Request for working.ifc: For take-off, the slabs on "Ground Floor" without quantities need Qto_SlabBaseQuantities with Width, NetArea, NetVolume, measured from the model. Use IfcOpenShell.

First a look at what the model holds.

```python
import ifcopenshell
import ifcopenshell.util.element
import ifcopenshell.util.unit

model = ifcopenshell.open("working.ifc")
print(model.schema)
for unit_type in ("LENGTHUNIT", "AREAUNIT", "VOLUMEUNIT"):
    print(unit_type, ifcopenshell.util.unit.calculate_unit_scale(model, unit_type))
storey = next(s for s in model.by_type("IfcBuildingStorey") if s.Name == "Ground Floor")
slabs = [e for e in ifcopenshell.util.element.get_decomposition(storey) if e.is_a("IfcSlab")]
for e in sorted(slabs, key=lambda e: e.id()):
    print(e.id(), e.is_a(), e.Name, list(ifcopenshell.util.element.get_psets(e, qtos_only=True)), sep=" | ")
```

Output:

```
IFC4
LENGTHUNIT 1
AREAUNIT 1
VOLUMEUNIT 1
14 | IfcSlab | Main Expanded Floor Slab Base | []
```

```python
import ifcopenshell
import ifcopenshell.api.pset
import ifcopenshell.geom
import ifcopenshell.util.element
import ifcopenshell.util.shape
import ifcopenshell.util.unit

model = ifcopenshell.open("working.ifc")
unit_scale = ifcopenshell.util.unit.calculate_unit_scale(model)
area_scale = ifcopenshell.util.unit.calculate_unit_scale(model, "AREAUNIT")
volume_scale = ifcopenshell.util.unit.calculate_unit_scale(model, "VOLUMEUNIT")
settings = ifcopenshell.geom.settings()

storey = next(s for s in model.by_type("IfcBuildingStorey") if s.Name == "Ground Floor")
slabs = [e for e in ifcopenshell.util.element.get_decomposition(storey) if e.is_a("IfcSlab")]

for e in sorted(slabs, key=lambda e: e.id()):
    if ifcopenshell.util.element.get_psets(e, qtos_only=True, should_inherit=False):
        continue
    # Geometry comes back in metres, in the element's own axes.
    shape = ifcopenshell.geom.create_shape(settings, e)
    values = {
        "Width": ifcopenshell.util.shape.get_z(shape.geometry) / unit_scale,
        "NetArea": ifcopenshell.util.shape.get_footprint_area(shape.geometry) / area_scale,
        "NetVolume": ifcopenshell.util.shape.get_volume(shape.geometry) / volume_scale,
    }
    qto = ifcopenshell.api.pset.add_qto(model, product=e, name="Qto_SlabBaseQuantities")
    ifcopenshell.api.pset.edit_qto(model, qto=qto, properties=values)
    print(e.id(), {k: round(v, 3) for k, v in values.items()})

model.write("working_updated.ifc")
```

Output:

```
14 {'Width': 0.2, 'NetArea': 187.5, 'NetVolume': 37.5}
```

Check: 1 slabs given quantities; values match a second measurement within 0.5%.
